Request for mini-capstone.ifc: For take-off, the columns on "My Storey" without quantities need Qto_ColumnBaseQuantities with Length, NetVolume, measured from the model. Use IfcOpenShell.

First a look at what the model holds.

```python
import ifcopenshell
import ifcopenshell.util.element
import ifcopenshell.util.unit

model = ifcopenshell.open("mini-capstone.ifc")
print(model.schema)
for unit_type in ("LENGTHUNIT", "AREAUNIT", "VOLUMEUNIT"):
    print(unit_type, ifcopenshell.util.unit.calculate_unit_scale(model, unit_type))
storey = next(s for s in model.by_type("IfcBuildingStorey") if s.Name == "My Storey")
columns = [e for e in ifcopenshell.util.element.get_decomposition(storey) if e.is_a("IfcColumn")]
for e in sorted(columns, key=lambda e: e.id()):
    print(e.id(), e.is_a(), e.Name, list(ifcopenshell.util.element.get_psets(e, qtos_only=True)), sep=" | ")
```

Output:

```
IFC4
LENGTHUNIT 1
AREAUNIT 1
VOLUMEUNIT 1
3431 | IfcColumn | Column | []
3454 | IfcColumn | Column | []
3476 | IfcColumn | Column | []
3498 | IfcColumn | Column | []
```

```python
import ifcopenshell
import ifcopenshell.api.pset
import ifcopenshell.geom
import ifcopenshell.util.element
import ifcopenshell.util.shape
import ifcopenshell.util.unit

model = ifcopenshell.open("mini-capstone.ifc")
unit_scale = ifcopenshell.util.unit.calculate_unit_scale(model)
volume_scale = ifcopenshell.util.unit.calculate_unit_scale(model, "VOLUMEUNIT")
settings = ifcopenshell.geom.settings()

storey = next(s for s in model.by_type("IfcBuildingStorey") if s.Name == "My Storey")
columns = [e for e in ifcopenshell.util.element.get_decomposition(storey) if e.is_a("IfcColumn")]

for e in sorted(columns, key=lambda e: e.id()):
    if ifcopenshell.util.element.get_psets(e, qtos_only=True, should_inherit=False):
        continue
    # Geometry comes back in metres, in the element's own axes.
    shape = ifcopenshell.geom.create_shape(settings, e)
    values = {
        "Length": ifcopenshell.util.shape.get_z(shape.geometry) / unit_scale,
        "NetVolume": ifcopenshell.util.shape.get_volume(shape.geometry) / volume_scale,
    }
    qto = ifcopenshell.api.pset.add_qto(model, product=e, name="Qto_ColumnBaseQuantities")
    ifcopenshell.api.pset.edit_qto(model, qto=qto, properties=values)
    print(e.id(), {k: round(v, 3) for k, v in values.items()})

model.write("mini-capstone_updated.ifc")
```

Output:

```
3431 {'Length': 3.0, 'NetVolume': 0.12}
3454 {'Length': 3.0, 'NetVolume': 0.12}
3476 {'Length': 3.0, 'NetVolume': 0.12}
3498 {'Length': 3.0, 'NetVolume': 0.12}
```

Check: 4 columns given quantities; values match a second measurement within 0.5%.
